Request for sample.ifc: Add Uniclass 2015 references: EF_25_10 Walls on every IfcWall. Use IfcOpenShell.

First a look at what the model holds.

```python
import ifcopenshell

model = ifcopenshell.open("sample.ifc")
print(model.schema)
print("classifications:", [c.Name for c in model.by_type("IfcClassification")])
for ifc_class in ("IfcDoor", "IfcRoof", "IfcStair", "IfcWall", "IfcWindow"):
    print(ifc_class, len(model.by_type(ifc_class)))
```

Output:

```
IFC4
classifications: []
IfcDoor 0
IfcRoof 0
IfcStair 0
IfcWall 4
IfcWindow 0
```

```python
import ifcopenshell
import ifcopenshell.api.classification

model = ifcopenshell.open("sample.ifc")

system = ifcopenshell.api.classification.add_classification(model, classification="Uniclass 2015")

codes = {
    "IfcWall": ("EF_25_10", "Walls"),
}
for ifc_class, (code, name) in codes.items():
    products = model.by_type(ifc_class)
    ifcopenshell.api.classification.add_reference(
        model, products=products, classification=system, identification=code, name=name
    )
    print(code, len(products))

model.write("sample_updated.ifc")
```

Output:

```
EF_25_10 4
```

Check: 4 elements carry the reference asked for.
